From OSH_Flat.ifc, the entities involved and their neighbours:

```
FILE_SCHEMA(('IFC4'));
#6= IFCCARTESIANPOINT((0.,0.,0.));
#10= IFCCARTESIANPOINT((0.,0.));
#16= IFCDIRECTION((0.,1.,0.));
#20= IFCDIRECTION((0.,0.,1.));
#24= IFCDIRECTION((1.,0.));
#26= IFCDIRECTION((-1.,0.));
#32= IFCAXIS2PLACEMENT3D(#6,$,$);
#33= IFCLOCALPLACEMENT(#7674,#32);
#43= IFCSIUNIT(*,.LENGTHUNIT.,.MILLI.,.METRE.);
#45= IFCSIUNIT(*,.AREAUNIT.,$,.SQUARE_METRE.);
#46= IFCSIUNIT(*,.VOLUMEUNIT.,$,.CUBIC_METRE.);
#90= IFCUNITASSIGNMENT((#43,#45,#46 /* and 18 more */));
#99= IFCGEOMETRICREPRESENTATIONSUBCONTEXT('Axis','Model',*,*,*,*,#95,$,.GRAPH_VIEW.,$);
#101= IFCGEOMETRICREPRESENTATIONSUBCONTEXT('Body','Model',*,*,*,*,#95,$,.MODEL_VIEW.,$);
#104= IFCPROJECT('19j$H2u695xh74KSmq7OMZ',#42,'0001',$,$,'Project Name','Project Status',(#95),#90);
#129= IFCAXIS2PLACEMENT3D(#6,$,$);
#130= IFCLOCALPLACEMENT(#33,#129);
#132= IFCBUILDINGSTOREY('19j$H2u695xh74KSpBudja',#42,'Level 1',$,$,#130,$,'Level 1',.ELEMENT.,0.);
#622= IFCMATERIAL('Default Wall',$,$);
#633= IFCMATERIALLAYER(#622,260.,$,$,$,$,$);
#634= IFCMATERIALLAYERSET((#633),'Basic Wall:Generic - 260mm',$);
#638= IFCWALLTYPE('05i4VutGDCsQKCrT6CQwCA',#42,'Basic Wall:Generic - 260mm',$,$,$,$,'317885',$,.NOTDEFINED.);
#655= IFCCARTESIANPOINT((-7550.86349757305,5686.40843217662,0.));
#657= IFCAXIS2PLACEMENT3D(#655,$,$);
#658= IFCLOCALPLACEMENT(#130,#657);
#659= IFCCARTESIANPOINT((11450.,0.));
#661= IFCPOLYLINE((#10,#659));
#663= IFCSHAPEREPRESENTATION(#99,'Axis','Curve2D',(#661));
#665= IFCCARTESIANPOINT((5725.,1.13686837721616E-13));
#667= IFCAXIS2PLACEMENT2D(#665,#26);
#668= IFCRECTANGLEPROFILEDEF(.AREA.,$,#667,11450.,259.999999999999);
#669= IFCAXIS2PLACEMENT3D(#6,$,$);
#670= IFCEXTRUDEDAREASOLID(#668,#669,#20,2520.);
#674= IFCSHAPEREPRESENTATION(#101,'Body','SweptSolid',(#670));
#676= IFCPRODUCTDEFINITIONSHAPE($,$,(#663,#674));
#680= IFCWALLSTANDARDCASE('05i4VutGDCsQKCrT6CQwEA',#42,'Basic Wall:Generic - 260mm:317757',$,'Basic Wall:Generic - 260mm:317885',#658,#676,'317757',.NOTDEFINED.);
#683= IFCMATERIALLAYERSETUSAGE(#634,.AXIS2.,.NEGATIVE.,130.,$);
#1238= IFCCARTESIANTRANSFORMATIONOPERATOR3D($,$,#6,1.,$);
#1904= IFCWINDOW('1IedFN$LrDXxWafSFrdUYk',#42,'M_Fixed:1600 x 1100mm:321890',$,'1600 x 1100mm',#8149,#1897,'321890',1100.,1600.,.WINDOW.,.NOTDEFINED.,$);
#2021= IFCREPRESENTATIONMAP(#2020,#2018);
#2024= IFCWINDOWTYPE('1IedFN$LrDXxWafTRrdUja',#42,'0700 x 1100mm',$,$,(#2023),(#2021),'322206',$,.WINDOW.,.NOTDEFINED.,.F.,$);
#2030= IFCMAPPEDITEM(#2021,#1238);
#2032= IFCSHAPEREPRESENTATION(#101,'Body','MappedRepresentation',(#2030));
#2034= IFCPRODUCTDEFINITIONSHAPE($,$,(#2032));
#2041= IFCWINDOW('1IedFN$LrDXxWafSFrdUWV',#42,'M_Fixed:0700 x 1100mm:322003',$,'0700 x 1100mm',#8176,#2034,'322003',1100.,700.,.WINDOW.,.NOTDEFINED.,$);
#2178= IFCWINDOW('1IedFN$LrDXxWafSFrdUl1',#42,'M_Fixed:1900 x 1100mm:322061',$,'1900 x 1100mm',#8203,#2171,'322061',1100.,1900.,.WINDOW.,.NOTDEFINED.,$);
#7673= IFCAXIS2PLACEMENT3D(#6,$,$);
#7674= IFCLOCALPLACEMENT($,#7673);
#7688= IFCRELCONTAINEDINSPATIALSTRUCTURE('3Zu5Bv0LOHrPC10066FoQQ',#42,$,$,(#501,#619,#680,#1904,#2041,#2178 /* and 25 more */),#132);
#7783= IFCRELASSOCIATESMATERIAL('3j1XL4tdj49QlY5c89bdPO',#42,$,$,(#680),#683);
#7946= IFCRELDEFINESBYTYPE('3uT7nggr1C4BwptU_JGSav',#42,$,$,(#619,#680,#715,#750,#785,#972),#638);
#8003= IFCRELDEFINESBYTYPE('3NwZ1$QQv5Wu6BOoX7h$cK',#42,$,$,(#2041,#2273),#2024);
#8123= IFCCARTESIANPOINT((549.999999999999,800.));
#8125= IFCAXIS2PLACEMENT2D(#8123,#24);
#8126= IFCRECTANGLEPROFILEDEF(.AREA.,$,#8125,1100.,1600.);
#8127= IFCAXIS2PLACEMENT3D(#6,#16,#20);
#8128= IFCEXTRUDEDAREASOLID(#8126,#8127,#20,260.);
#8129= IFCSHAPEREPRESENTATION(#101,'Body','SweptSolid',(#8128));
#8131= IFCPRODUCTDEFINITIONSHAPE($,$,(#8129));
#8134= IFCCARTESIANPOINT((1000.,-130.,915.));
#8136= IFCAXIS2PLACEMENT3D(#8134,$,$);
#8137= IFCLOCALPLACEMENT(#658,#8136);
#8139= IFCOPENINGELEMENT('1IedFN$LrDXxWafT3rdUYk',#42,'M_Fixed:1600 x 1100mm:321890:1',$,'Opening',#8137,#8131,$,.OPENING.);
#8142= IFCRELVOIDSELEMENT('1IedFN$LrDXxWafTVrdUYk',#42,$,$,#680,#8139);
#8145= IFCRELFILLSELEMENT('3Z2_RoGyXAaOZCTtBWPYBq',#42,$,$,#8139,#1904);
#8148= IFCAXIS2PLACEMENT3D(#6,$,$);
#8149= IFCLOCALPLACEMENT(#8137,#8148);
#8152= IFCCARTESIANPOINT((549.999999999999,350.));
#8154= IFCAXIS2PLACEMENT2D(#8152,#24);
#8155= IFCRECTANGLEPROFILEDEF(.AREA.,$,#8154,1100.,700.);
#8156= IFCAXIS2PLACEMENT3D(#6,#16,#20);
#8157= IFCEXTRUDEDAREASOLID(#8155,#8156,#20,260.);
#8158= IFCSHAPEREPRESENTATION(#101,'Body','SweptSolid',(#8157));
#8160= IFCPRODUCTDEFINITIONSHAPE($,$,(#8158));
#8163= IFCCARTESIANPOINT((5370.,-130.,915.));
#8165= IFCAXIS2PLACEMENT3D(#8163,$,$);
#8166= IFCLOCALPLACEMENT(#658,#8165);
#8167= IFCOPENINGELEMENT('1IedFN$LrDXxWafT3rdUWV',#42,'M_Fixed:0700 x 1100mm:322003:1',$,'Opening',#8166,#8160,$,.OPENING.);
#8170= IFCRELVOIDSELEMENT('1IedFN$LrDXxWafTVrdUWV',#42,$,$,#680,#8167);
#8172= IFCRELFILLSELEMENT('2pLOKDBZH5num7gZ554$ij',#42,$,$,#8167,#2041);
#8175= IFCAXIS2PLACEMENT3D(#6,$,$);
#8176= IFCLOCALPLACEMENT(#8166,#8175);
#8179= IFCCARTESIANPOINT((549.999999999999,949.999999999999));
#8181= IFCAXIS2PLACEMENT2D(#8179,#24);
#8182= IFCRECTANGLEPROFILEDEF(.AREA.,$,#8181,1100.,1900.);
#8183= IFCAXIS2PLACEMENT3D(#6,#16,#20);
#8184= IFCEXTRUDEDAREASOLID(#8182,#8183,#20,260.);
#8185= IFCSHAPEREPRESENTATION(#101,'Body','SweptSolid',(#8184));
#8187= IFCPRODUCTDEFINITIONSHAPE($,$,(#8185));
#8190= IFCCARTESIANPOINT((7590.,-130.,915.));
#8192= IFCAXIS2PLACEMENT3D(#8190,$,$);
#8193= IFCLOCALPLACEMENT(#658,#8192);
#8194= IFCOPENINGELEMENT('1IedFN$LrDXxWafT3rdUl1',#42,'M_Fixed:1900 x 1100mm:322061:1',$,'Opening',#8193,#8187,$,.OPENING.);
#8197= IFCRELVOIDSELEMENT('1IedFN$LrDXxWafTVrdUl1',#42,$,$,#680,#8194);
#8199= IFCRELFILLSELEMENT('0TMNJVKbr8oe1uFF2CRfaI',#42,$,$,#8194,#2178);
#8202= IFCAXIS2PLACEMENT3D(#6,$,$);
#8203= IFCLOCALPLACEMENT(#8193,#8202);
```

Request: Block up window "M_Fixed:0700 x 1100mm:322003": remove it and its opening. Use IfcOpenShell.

```python
import ifcopenshell
import ifcopenshell.api.feature
import ifcopenshell.api.root
import ifcopenshell.geom
import ifcopenshell.util.shape

model = ifcopenshell.open("OSH_Flat.ifc")
settings = ifcopenshell.geom.settings()


def volume(element):
    """Net volume in cubic metres, openings subtracted."""
    shape = ifcopenshell.geom.create_shape(settings, element)
    return ifcopenshell.util.shape.get_volume(shape.geometry)


window = model.by_guid("1IedFN$LrDXxWafSFrdUWV")
opening = window.FillsVoids[0].RelatingOpeningElement
wall = opening.VoidsElements[0].RelatingBuildingElement
before = volume(wall)

ifcopenshell.api.root.remove_product(model, product=window)
ifcopenshell.api.feature.remove_feature(model, feature=opening)

after = volume(wall)

print(f"wall volume {before:.3f} -> {after:.3f} m3")

model.write("OSH_Flat_rev.ifc")
```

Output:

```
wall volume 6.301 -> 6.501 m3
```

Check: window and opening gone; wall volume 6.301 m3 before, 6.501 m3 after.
